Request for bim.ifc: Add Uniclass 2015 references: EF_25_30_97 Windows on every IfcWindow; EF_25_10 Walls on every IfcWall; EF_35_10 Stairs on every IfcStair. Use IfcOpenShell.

First a look at what the model holds.

```python
import ifcopenshell

model = ifcopenshell.open("bim.ifc")
print(model.schema)
print("classifications:", [c.Name for c in model.by_type("IfcClassification")])
for ifc_class in ("IfcDoor", "IfcRoof", "IfcStair", "IfcWall", "IfcWindow"):
    print(ifc_class, len(model.by_type(ifc_class)))
```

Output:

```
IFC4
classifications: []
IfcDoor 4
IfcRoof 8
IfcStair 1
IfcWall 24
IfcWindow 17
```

```python
import ifcopenshell
import ifcopenshell.api.classification

model = ifcopenshell.open("bim.ifc")

system = ifcopenshell.api.classification.add_classification(model, classification="Uniclass 2015")

codes = {
    "IfcWindow": ("EF_25_30_97", "Windows"),
    "IfcWall": ("EF_25_10", "Walls"),
    "IfcStair": ("EF_35_10", "Stairs"),
}
for ifc_class, (code, name) in codes.items():
    products = model.by_type(ifc_class)
    ifcopenshell.api.classification.add_reference(
        model, products=products, classification=system, identification=code, name=name
    )
    print(code, len(products))

model.write("bim_rev.ifc")
```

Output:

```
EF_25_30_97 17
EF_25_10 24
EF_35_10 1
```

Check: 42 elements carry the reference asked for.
